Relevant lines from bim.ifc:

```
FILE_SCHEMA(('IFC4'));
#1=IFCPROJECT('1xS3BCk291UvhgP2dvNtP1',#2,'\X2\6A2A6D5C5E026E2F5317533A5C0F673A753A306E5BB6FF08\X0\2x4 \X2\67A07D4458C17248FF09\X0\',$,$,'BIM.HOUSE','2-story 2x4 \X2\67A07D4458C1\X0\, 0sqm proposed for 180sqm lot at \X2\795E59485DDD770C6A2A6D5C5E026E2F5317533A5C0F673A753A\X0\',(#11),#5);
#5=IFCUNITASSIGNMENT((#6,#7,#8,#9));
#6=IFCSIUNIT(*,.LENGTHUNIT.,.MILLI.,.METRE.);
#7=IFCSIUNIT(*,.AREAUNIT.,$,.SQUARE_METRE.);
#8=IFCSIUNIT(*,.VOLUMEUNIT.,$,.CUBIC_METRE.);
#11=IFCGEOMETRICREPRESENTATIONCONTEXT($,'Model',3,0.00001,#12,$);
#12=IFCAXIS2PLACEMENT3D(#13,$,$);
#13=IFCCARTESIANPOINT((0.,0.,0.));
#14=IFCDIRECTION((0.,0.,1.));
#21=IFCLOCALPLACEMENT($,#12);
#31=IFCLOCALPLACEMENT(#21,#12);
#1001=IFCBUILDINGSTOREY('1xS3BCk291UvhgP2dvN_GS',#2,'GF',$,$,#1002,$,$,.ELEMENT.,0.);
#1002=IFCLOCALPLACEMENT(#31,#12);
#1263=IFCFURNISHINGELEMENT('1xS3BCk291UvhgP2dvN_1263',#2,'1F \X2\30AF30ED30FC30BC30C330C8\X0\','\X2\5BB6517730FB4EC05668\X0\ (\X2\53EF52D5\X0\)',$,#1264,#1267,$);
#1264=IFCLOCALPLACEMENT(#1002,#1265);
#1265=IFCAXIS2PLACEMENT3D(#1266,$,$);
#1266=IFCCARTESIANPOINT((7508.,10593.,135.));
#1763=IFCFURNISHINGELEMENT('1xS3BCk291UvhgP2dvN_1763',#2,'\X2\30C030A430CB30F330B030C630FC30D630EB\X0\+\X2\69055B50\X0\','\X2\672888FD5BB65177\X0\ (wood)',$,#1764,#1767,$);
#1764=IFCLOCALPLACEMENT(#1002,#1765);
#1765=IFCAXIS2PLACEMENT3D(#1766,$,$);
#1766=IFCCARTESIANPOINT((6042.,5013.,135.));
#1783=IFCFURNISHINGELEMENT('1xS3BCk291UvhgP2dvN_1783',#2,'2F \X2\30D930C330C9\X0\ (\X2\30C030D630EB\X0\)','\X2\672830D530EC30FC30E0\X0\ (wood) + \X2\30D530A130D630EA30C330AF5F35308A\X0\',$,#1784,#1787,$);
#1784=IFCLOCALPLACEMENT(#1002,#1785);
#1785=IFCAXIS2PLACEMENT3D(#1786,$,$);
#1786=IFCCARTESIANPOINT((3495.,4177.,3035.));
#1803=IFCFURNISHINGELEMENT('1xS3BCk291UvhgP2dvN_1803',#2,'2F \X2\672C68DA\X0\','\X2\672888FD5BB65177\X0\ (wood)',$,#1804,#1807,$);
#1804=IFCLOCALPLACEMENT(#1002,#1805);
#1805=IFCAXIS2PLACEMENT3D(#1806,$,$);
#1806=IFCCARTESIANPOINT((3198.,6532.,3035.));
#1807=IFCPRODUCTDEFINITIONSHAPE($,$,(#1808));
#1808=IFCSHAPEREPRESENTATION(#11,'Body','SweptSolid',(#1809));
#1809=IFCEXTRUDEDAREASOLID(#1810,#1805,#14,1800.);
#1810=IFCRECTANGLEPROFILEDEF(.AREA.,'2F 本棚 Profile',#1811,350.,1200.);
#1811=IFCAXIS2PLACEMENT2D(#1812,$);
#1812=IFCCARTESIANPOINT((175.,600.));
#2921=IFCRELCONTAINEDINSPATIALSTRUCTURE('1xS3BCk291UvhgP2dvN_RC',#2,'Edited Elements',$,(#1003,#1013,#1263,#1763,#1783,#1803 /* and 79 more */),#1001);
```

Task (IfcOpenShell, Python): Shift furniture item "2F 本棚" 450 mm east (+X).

```python
import ifcopenshell
import ifcopenshell.api.geometry
import ifcopenshell.util.placement
import ifcopenshell.util.unit

model = ifcopenshell.open("bim.ifc")
unit_scale = ifcopenshell.util.unit.calculate_unit_scale(model)

item = model.by_guid("1xS3BCk291UvhgP2dvN_1803")
matrix = ifcopenshell.util.placement.get_local_placement(item.ObjectPlacement)
matrix[0, 3] += 0.45 / unit_scale
ifcopenshell.api.geometry.edit_object_placement(model, product=item, matrix=matrix, is_si=False)

print(ifcopenshell.util.placement.get_local_placement(item.ObjectPlacement).round(3) + 0.0)

model.write("bim_v2.ifc")
```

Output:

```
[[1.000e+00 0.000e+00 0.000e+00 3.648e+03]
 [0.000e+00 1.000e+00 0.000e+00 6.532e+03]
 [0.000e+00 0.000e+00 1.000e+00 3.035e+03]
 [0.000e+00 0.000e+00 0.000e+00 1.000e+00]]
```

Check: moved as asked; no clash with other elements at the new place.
